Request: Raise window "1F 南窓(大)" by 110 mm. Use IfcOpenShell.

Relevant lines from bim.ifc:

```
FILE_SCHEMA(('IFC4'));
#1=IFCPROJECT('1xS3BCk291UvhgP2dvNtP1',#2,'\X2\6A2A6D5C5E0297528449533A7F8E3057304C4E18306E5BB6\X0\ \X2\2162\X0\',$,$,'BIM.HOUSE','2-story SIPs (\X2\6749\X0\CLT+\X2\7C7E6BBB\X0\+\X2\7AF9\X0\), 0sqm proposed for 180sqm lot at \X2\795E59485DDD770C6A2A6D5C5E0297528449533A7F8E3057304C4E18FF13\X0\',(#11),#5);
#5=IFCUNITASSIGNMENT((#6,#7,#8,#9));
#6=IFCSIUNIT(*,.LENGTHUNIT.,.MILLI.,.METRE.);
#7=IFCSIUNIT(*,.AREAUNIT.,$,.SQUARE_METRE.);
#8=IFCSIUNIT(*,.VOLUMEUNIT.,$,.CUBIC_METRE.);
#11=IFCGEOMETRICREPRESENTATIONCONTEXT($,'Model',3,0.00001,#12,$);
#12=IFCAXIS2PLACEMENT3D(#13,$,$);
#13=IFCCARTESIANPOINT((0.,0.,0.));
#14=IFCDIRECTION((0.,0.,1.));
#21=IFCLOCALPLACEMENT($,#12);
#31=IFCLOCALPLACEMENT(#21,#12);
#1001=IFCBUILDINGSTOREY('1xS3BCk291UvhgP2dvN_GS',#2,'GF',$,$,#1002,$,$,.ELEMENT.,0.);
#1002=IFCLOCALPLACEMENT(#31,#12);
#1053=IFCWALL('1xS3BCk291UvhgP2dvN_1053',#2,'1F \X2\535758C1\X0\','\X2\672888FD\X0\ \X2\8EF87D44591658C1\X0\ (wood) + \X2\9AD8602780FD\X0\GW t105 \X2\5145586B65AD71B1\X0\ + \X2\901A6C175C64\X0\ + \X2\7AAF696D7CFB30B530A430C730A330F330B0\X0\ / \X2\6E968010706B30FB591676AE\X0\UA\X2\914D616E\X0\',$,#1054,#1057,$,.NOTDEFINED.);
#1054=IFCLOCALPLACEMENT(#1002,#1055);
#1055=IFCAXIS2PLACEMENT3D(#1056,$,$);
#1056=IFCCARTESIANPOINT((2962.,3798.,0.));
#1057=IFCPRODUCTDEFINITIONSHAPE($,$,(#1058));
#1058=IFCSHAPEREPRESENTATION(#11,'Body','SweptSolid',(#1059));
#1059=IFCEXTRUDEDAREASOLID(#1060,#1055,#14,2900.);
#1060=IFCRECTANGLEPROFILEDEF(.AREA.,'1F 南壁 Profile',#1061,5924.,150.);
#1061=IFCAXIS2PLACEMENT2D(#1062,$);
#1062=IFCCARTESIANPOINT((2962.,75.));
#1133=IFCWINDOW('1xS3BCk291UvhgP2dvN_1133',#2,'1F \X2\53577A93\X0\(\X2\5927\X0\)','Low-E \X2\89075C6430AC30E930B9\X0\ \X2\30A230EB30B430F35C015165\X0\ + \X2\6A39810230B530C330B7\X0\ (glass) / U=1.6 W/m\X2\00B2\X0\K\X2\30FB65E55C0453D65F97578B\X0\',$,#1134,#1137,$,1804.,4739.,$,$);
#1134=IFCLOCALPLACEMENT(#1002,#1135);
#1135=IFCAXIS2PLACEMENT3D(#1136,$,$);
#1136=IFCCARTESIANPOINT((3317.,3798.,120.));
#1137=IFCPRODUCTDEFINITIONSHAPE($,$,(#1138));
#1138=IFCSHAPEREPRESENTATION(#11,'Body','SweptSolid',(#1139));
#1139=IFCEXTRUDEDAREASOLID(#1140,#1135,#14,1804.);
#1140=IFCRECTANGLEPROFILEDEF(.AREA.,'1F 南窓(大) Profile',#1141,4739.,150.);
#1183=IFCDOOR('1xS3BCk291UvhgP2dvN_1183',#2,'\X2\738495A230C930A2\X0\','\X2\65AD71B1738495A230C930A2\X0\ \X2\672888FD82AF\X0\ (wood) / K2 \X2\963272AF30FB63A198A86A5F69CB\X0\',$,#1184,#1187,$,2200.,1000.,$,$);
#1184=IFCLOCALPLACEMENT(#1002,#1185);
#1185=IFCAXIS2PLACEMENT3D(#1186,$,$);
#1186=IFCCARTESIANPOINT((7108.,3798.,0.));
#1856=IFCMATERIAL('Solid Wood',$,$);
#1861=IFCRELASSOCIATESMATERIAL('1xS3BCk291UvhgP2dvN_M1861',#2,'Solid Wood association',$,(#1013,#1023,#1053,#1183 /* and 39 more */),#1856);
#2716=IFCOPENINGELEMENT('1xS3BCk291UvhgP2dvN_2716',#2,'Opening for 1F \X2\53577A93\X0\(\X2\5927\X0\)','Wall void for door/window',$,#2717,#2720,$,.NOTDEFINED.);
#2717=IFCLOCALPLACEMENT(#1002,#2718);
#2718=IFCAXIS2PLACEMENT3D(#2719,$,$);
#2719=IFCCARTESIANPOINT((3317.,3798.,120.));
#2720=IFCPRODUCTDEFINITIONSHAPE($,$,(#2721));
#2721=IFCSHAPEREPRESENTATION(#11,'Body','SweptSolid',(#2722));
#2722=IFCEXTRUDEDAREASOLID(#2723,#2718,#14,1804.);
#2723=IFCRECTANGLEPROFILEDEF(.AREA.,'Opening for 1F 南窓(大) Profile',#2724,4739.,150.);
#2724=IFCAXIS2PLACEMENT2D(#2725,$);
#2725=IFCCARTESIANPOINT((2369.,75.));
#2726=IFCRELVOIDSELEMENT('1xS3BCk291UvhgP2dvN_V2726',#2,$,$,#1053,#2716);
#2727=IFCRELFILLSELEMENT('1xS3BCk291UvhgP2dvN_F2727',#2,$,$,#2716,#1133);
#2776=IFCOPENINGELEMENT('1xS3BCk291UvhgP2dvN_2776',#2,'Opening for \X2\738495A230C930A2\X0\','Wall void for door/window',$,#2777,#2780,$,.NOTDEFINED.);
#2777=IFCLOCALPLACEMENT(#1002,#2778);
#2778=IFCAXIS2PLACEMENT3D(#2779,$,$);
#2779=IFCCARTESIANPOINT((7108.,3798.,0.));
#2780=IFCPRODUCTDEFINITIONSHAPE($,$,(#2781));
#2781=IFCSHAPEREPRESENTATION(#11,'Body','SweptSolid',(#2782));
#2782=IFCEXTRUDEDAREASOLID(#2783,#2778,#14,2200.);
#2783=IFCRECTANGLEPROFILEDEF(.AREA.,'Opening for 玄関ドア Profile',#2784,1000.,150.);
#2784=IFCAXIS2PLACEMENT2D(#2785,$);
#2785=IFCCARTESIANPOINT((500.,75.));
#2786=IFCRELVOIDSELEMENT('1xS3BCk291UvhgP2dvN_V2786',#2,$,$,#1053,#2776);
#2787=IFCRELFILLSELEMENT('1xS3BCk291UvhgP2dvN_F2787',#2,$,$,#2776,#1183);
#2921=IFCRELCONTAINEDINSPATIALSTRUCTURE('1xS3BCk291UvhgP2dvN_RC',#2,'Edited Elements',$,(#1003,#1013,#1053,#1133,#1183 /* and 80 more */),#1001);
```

```python
import numpy as np
import ifcopenshell
import ifcopenshell.api.geometry
import ifcopenshell.util.placement
import ifcopenshell.util.unit

model = ifcopenshell.open("bim.ifc")
unit_scale = ifcopenshell.util.unit.calculate_unit_scale(model)

window = model.by_guid("1xS3BCk291UvhgP2dvN_1133")
opening = window.FillsVoids[0].RelatingOpeningElement
dz = 0.11 / unit_scale

shift = np.array([0.0, 0.0, dz])
# The window is not placed relative to its opening, so move both.
for product in (opening, window):
    matrix = ifcopenshell.util.placement.get_local_placement(product.ObjectPlacement)
    matrix[:3, 3] += shift
    ifcopenshell.api.geometry.edit_object_placement(model, product=product, matrix=matrix, is_si=False)

print(f"moved by {dz * unit_scale:+.3f} m")

model.write("bim-out.ifc")
```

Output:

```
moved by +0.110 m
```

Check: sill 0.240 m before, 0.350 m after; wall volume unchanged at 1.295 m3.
